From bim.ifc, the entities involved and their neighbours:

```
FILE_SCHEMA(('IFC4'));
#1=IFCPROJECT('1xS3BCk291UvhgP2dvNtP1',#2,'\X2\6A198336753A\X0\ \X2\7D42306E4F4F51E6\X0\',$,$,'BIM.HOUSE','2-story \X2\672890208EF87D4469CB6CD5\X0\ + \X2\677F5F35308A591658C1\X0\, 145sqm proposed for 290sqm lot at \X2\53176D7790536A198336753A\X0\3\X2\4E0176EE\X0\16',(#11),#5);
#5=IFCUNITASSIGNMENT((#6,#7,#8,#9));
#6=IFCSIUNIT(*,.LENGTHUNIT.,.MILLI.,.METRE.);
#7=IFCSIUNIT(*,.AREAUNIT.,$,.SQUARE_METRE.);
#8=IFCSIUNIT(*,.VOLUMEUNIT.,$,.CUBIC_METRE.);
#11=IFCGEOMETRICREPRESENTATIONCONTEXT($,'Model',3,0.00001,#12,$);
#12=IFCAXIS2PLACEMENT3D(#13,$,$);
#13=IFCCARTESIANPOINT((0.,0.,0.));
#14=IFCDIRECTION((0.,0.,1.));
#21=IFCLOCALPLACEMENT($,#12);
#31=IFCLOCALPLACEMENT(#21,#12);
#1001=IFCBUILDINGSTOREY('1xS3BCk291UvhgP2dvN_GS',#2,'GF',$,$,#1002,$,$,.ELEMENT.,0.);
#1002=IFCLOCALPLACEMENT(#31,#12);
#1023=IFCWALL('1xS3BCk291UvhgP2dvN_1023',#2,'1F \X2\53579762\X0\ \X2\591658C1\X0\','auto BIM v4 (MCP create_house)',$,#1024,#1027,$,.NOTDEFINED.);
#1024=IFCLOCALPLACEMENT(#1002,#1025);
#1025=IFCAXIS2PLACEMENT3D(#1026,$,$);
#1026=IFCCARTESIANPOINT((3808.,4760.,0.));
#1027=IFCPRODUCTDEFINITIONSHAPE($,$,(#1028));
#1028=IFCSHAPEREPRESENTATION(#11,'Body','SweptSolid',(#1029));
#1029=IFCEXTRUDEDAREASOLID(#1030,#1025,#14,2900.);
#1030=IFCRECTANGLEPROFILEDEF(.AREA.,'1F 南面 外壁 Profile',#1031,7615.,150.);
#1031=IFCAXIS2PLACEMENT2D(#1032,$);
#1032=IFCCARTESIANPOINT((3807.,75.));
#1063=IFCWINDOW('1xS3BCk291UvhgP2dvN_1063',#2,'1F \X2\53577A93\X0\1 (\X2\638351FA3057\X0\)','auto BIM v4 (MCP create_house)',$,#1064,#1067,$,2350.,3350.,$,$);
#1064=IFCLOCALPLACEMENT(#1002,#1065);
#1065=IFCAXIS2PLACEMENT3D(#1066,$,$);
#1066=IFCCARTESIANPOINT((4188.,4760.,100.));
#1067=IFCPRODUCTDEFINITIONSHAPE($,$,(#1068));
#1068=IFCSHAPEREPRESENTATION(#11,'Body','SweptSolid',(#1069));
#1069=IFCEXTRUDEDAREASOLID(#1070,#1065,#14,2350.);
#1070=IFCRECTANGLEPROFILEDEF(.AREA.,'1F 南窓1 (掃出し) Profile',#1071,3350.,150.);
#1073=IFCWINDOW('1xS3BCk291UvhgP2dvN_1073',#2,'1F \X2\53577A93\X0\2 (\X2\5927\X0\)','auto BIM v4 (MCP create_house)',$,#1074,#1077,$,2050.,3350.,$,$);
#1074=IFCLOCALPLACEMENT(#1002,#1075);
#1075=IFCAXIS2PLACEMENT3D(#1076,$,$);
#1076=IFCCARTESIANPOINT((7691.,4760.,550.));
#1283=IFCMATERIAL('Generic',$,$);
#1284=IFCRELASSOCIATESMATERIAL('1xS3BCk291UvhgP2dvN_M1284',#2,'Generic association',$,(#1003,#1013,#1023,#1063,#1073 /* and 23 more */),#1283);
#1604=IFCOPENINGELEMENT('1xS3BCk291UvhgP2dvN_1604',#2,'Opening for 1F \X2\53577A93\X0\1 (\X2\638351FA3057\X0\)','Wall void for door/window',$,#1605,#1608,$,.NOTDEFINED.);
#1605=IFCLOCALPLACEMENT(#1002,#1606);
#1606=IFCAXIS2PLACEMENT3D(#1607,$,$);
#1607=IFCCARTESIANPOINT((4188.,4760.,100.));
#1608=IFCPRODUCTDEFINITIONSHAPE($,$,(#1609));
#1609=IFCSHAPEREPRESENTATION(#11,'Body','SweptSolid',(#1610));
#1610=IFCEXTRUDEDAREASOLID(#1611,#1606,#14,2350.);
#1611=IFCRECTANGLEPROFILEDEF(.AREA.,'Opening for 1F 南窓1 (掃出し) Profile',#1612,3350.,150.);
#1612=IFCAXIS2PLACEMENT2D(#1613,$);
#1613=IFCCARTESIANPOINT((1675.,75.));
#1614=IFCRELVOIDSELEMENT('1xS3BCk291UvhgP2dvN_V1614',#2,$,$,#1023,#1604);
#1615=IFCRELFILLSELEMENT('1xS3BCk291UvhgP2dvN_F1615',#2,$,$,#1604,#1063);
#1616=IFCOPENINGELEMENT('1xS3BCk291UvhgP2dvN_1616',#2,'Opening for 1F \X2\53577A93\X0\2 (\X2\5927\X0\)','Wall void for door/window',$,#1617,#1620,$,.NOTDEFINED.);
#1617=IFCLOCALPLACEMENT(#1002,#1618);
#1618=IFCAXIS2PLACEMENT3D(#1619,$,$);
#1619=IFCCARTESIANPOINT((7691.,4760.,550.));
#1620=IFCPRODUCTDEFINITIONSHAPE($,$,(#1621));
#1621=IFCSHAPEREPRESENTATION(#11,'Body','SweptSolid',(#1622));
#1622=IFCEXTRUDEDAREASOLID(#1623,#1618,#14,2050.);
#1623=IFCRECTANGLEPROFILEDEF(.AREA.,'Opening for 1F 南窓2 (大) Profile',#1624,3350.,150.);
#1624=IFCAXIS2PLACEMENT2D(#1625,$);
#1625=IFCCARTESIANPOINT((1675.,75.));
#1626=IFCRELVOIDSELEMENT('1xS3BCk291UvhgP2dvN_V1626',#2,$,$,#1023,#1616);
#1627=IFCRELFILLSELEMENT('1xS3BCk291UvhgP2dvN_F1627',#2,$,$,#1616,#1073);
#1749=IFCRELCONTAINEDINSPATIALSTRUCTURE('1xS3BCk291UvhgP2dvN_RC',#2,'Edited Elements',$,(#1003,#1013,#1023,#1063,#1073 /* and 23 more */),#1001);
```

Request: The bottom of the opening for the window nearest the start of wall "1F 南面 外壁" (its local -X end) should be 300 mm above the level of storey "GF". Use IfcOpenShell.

```python
import numpy as np
import ifcopenshell
import ifcopenshell.api.geometry
import ifcopenshell.geom
import ifcopenshell.util.element
import ifcopenshell.util.placement
import ifcopenshell.util.shape
import ifcopenshell.util.unit

model = ifcopenshell.open("bim.ifc")
unit_scale = ifcopenshell.util.unit.calculate_unit_scale(model)

window = model.by_guid("1xS3BCk291UvhgP2dvN_1063")
opening = window.FillsVoids[0].RelatingOpeningElement
storey = ifcopenshell.util.element.get_container(window, ifc_class="IfcBuildingStorey")
level = ifcopenshell.util.placement.get_local_placement(storey.ObjectPlacement)[2, 3]

# The opening's origin need not be at the sill, so measure its lowest point.
shape = ifcopenshell.geom.create_shape(ifcopenshell.geom.settings(), opening)
bottom = ifcopenshell.util.shape.get_shape_bottom_elevation(shape, shape.geometry) / unit_scale
dz = level + 0.3 / unit_scale - bottom

shift = np.array([0.0, 0.0, dz])
# The window is not placed relative to its opening, so move both.
for product in (opening, window):
    matrix = ifcopenshell.util.placement.get_local_placement(product.ObjectPlacement)
    matrix[:3, 3] += shift
    ifcopenshell.api.geometry.edit_object_placement(model, product=product, matrix=matrix, is_si=False)

print(f"moved by {dz * unit_scale:+.3f} m")

model.write("bim-out.ifc")
```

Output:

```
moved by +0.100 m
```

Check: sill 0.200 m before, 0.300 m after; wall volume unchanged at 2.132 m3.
